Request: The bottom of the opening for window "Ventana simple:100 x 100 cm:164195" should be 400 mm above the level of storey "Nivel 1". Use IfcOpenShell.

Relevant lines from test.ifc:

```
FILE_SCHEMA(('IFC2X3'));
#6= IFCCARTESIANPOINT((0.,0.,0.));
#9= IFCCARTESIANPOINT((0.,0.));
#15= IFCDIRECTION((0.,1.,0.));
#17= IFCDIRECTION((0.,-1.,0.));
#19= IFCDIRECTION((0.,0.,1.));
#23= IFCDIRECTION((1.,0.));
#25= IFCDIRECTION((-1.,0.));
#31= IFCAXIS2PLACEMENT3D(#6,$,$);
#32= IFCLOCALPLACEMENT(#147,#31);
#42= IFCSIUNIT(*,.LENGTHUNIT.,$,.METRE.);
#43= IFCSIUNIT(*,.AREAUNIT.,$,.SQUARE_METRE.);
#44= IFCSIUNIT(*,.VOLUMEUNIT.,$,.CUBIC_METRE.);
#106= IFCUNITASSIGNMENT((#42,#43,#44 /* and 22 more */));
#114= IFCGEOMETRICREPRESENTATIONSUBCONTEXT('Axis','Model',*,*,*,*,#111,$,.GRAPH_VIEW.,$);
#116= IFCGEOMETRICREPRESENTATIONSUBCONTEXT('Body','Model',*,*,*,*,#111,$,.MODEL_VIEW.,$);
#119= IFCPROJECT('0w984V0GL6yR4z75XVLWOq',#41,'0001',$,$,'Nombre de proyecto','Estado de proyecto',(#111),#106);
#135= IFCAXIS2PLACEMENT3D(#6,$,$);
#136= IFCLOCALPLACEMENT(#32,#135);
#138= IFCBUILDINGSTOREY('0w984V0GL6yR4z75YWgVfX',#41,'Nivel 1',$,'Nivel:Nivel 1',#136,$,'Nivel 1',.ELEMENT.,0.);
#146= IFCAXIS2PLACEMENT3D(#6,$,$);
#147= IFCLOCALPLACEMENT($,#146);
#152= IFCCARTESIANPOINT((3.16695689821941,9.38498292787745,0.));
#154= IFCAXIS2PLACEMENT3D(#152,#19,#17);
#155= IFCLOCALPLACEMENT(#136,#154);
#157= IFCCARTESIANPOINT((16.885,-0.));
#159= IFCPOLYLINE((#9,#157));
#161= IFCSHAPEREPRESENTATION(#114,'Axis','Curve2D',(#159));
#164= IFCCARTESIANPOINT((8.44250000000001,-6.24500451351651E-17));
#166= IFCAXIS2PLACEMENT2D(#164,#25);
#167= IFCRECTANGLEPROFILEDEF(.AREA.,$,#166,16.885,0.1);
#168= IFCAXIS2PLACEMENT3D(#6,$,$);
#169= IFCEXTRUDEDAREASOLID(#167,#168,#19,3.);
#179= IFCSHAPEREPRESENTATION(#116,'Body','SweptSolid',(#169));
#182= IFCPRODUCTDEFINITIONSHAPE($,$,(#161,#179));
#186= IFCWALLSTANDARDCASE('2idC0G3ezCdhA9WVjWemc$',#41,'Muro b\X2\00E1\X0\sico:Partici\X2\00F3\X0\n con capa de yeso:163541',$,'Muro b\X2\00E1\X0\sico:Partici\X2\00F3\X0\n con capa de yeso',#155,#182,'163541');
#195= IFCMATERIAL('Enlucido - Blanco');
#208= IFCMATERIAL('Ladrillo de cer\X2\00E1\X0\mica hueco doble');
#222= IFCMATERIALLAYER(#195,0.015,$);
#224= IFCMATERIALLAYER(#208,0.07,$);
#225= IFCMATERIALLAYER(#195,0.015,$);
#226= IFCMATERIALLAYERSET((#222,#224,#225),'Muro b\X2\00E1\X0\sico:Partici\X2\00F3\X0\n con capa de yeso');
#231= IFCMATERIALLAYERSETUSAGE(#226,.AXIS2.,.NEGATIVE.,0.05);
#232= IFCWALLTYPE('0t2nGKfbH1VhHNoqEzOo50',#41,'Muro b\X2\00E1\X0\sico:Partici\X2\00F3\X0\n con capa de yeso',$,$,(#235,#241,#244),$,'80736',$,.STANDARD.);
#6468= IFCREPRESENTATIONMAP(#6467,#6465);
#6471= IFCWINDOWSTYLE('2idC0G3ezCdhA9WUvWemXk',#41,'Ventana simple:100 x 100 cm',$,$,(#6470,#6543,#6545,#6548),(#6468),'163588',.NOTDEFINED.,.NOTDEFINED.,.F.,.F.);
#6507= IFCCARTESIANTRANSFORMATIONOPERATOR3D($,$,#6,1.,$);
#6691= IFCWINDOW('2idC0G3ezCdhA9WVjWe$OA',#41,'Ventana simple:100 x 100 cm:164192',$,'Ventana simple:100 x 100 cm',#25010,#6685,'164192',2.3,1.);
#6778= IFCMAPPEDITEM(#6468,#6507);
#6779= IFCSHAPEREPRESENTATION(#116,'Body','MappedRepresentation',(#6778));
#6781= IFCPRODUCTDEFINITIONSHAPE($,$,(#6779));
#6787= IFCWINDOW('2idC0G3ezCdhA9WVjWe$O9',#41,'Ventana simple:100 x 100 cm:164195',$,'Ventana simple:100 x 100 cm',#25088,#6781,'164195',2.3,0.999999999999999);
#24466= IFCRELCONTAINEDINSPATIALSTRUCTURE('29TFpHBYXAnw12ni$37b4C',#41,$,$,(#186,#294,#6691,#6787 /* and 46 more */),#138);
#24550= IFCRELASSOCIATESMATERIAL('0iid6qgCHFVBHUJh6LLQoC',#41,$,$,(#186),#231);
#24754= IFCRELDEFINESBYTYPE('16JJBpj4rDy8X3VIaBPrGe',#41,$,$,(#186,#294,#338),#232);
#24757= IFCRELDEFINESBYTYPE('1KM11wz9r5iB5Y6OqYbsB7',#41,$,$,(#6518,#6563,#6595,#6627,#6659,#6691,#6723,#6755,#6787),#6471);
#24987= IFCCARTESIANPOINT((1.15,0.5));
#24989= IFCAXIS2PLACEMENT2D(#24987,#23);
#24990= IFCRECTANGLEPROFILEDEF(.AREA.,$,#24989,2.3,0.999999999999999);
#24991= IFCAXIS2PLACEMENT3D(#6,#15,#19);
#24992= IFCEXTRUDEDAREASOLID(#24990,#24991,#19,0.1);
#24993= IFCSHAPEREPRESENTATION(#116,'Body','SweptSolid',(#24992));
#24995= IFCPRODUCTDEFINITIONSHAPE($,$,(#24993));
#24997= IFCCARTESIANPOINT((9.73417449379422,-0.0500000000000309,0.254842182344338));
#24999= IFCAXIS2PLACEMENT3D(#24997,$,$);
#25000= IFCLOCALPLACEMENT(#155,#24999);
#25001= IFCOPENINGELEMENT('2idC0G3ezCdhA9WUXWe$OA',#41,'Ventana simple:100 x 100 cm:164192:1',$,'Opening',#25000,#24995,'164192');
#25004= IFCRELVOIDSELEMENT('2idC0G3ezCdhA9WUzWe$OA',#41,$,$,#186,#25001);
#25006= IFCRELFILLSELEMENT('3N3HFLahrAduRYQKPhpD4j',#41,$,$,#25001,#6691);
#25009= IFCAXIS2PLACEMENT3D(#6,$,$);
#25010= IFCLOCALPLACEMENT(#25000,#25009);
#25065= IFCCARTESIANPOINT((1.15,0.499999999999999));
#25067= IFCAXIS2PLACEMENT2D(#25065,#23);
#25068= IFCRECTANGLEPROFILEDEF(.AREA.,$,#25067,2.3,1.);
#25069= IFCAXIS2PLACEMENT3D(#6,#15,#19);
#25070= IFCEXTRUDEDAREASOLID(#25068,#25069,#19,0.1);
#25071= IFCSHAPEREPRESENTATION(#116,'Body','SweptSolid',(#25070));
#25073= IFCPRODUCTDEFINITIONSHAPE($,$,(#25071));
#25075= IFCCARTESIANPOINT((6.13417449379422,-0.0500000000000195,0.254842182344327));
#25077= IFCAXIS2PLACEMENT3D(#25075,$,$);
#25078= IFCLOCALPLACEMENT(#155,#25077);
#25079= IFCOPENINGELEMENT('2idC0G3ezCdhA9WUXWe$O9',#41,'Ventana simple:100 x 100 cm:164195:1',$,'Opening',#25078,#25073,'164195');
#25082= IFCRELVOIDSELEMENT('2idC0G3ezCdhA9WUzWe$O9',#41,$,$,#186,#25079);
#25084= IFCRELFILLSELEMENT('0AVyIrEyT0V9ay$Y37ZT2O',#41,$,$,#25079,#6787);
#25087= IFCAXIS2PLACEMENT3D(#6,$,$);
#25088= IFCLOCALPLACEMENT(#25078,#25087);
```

```python
import numpy as np
import ifcopenshell
import ifcopenshell.api.geometry
import ifcopenshell.geom
import ifcopenshell.util.element
import ifcopenshell.util.placement
import ifcopenshell.util.shape
import ifcopenshell.util.unit

model = ifcopenshell.open("test.ifc")
unit_scale = ifcopenshell.util.unit.calculate_unit_scale(model)

window = model.by_id(6787)
opening = window.FillsVoids[0].RelatingOpeningElement
storey = ifcopenshell.util.element.get_container(window, ifc_class="IfcBuildingStorey")
level = ifcopenshell.util.placement.get_local_placement(storey.ObjectPlacement)[2, 3]

# The opening's origin need not be at the sill, so measure its lowest point.
shape = ifcopenshell.geom.create_shape(ifcopenshell.geom.settings(), opening)
bottom = ifcopenshell.util.shape.get_shape_bottom_elevation(shape, shape.geometry) / unit_scale
dz = level + 0.4 / unit_scale - bottom

shift = np.array([0.0, 0.0, dz])
# The window is placed relative to its opening, so it follows when the opening moves.
matrix = ifcopenshell.util.placement.get_local_placement(opening.ObjectPlacement)
matrix[:3, 3] += shift
ifcopenshell.api.geometry.edit_object_placement(
    model, product=opening, matrix=matrix, is_si=False, should_transform_children=True
)

print(f"moved by {dz * unit_scale:+.3f} m")

model.write("test-out.ifc")
```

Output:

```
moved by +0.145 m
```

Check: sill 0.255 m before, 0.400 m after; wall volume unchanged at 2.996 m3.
